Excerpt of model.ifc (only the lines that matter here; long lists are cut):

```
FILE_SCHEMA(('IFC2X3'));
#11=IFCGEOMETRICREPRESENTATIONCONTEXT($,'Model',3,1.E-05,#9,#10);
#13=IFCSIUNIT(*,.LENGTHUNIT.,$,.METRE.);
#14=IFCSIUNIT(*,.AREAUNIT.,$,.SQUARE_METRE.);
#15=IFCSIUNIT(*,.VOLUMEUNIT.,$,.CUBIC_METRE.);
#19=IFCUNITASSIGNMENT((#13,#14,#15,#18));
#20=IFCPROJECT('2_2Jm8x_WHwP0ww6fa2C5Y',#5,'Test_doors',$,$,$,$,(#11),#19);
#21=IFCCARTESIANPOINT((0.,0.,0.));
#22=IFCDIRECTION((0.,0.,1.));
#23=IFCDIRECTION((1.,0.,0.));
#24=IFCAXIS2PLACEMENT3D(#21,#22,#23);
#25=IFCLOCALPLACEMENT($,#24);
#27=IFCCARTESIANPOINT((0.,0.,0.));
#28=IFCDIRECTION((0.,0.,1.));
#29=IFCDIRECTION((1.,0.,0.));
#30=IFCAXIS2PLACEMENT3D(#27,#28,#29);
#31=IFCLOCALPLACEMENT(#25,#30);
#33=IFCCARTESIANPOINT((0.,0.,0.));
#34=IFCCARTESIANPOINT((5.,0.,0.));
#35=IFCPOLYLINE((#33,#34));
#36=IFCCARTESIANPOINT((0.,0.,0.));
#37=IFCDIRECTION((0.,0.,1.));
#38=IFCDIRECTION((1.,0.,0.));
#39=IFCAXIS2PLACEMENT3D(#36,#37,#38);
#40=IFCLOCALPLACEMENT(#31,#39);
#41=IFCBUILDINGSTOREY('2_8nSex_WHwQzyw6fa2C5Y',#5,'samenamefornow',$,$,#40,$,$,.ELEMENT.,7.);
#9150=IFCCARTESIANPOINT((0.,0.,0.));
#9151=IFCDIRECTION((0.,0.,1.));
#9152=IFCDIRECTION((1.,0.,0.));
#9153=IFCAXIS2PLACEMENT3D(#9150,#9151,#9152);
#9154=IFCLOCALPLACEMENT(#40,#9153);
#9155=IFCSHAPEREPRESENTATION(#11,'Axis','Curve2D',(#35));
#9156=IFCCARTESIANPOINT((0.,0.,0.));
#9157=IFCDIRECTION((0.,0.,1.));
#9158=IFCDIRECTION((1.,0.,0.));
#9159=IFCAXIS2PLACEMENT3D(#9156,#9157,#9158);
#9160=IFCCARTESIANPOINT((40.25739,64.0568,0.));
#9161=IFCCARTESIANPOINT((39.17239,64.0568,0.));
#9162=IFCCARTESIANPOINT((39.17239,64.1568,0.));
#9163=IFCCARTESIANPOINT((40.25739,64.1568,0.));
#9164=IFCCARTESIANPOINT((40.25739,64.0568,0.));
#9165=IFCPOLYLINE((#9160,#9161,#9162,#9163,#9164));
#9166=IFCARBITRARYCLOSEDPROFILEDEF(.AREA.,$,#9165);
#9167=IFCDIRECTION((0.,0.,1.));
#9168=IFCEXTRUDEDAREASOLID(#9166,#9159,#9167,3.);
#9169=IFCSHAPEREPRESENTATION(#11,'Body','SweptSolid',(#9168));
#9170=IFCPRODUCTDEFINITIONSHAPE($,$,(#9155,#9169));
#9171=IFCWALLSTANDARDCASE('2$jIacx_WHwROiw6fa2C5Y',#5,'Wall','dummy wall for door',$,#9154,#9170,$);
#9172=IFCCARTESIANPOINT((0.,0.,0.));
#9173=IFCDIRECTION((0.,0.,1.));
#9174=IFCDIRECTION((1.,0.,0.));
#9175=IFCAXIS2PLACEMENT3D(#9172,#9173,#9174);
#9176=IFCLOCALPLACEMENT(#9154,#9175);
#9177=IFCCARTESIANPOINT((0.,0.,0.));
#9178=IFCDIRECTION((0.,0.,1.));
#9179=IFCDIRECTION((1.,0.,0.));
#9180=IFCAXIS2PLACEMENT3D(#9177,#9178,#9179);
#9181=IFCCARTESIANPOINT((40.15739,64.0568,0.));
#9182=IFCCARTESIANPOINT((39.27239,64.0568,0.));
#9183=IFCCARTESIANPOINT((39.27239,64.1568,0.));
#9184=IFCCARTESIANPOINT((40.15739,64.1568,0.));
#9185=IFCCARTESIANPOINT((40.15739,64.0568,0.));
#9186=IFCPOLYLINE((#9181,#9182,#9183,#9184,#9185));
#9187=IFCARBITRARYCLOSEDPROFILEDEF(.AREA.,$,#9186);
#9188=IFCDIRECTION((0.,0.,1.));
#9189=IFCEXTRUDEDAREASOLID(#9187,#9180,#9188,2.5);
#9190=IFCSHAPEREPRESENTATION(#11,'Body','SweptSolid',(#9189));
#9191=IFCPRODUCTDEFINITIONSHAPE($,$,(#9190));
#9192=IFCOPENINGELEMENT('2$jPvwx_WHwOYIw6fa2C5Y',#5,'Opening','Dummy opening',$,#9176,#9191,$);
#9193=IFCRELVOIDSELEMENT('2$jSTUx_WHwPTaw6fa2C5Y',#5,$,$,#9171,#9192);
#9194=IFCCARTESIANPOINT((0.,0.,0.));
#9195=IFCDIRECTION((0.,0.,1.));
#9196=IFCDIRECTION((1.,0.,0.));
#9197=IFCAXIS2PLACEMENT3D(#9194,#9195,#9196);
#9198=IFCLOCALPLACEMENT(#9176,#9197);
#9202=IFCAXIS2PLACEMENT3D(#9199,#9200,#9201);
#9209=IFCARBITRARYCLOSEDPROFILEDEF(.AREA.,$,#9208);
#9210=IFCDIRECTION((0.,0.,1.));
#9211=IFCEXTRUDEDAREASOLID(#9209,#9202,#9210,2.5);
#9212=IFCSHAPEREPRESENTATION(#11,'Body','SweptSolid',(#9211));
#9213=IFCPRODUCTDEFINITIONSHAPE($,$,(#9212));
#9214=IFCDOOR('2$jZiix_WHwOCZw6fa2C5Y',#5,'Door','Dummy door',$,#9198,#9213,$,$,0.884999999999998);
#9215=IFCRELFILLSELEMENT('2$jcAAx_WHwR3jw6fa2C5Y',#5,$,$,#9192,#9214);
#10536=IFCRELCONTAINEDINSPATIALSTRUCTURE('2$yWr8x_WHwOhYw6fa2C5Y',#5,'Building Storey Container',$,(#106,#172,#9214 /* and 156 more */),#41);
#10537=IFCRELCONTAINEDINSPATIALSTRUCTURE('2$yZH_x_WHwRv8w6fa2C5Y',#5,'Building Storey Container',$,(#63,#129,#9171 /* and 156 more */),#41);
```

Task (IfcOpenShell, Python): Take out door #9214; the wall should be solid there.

```python
import ifcopenshell
import ifcopenshell.api.feature
import ifcopenshell.api.root
import ifcopenshell.geom
import ifcopenshell.util.shape

model = ifcopenshell.open("model.ifc")
settings = ifcopenshell.geom.settings()


def volume(element):
    """Net volume in cubic metres, openings subtracted."""
    shape = ifcopenshell.geom.create_shape(settings, element)
    return ifcopenshell.util.shape.get_volume(shape.geometry)


door = model.by_id(9214)
opening = door.FillsVoids[0].RelatingOpeningElement
wall = opening.VoidsElements[0].RelatingBuildingElement
before = volume(wall)

ifcopenshell.api.root.remove_product(model, product=door)
ifcopenshell.api.feature.remove_feature(model, feature=opening)

after = volume(wall)

print(f"wall volume {before:.3f} -> {after:.3f} m3")

model.write("model_rev.ifc")
```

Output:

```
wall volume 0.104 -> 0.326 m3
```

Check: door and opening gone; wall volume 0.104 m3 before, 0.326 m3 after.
